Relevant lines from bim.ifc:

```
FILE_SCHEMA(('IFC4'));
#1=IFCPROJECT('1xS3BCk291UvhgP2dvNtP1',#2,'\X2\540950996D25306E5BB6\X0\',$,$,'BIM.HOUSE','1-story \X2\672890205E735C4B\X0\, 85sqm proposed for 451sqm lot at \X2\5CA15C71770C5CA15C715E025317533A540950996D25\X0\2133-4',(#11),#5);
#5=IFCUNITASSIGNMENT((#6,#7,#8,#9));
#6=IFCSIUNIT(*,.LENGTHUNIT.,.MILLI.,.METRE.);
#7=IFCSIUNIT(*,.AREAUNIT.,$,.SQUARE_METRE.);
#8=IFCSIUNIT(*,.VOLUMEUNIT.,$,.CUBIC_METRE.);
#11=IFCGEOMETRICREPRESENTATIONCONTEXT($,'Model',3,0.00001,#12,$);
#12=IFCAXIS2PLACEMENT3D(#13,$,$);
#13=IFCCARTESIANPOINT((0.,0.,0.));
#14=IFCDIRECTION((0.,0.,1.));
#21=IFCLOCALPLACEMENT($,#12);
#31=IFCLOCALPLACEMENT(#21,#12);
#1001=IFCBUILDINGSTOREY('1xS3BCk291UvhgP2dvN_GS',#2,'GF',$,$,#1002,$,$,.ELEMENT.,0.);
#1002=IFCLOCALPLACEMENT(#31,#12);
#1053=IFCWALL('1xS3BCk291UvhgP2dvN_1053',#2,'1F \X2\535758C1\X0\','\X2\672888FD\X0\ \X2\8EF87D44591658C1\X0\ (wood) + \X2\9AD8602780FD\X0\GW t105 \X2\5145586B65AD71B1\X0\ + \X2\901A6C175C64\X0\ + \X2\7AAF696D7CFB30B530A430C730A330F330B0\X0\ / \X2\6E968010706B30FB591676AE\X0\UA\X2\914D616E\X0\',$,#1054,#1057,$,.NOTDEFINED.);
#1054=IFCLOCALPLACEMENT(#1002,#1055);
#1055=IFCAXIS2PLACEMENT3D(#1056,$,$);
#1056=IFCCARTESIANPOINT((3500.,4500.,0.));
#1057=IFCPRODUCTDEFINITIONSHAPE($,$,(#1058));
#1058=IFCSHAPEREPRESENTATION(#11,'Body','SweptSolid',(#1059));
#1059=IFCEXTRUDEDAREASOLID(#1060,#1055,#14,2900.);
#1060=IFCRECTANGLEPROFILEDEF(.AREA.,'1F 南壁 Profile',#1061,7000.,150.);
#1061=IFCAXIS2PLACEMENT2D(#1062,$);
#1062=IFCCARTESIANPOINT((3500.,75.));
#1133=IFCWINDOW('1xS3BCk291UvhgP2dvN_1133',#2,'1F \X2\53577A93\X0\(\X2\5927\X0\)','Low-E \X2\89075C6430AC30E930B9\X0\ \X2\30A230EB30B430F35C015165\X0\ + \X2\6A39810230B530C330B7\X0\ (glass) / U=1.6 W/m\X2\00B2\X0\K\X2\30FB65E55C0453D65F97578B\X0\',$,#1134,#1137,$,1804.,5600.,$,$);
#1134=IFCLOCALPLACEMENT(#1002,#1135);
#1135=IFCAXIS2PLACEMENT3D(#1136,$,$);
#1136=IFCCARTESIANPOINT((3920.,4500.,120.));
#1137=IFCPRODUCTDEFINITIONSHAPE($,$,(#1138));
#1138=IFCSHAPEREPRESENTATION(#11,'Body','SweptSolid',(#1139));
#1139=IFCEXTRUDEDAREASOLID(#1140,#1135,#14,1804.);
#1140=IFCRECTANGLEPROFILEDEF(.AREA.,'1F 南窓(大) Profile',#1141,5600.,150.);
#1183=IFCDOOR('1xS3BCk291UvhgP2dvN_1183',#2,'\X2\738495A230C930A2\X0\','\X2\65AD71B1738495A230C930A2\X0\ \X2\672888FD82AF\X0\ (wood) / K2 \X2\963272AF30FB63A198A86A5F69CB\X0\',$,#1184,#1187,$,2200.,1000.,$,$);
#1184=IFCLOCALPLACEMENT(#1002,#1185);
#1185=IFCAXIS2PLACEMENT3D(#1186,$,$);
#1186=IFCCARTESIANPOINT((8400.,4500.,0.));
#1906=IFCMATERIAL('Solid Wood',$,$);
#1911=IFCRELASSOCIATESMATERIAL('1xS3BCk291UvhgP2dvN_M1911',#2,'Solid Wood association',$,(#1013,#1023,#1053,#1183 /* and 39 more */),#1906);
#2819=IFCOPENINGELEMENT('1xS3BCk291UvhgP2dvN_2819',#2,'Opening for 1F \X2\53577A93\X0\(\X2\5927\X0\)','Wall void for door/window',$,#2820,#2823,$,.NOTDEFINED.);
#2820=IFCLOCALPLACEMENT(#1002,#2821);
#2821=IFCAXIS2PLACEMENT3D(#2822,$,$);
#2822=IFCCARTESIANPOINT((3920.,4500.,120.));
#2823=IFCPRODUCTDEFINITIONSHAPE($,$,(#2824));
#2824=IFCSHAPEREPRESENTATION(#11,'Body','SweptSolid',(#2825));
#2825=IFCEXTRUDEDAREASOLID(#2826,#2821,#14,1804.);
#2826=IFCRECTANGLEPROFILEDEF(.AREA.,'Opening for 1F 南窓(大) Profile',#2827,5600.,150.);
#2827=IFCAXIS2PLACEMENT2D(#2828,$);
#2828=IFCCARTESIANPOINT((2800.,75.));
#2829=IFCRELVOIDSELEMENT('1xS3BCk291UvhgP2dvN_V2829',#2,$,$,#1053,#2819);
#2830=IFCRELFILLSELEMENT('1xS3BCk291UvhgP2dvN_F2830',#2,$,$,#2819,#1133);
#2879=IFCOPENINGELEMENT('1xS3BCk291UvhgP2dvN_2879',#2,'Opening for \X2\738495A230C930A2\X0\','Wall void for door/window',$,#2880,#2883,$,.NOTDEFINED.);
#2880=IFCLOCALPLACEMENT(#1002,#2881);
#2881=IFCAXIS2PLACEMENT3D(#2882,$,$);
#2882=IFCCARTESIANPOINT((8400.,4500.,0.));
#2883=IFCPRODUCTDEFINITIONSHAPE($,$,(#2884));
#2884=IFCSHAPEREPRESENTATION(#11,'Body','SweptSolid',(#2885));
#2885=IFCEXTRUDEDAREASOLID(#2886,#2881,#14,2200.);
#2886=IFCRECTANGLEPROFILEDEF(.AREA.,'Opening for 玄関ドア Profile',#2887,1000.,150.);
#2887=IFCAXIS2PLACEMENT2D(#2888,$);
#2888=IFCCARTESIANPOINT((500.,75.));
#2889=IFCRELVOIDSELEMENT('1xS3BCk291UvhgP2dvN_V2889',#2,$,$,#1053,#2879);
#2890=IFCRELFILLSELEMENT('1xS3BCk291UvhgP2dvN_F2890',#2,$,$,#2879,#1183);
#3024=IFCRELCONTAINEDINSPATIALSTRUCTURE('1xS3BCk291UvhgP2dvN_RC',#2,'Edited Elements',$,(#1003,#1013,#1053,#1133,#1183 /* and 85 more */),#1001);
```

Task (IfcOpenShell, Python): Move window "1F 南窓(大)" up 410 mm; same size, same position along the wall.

```python
import numpy as np
import ifcopenshell
import ifcopenshell.api.geometry
import ifcopenshell.util.placement
import ifcopenshell.util.unit

model = ifcopenshell.open("bim.ifc")
unit_scale = ifcopenshell.util.unit.calculate_unit_scale(model)

window = model.by_id(1133)
opening = window.FillsVoids[0].RelatingOpeningElement
dz = 0.41 / unit_scale

shift = np.array([0.0, 0.0, dz])
# The window is not placed relative to its opening, so move both.
for product in (opening, window):
    matrix = ifcopenshell.util.placement.get_local_placement(product.ObjectPlacement)
    matrix[:3, 3] += shift
    ifcopenshell.api.geometry.edit_object_placement(model, product=product, matrix=matrix, is_si=False)

print(f"moved by {dz * unit_scale:+.3f} m")

model.write("bim-out.ifc")
```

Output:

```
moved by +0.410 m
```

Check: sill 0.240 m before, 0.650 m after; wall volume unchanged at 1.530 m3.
